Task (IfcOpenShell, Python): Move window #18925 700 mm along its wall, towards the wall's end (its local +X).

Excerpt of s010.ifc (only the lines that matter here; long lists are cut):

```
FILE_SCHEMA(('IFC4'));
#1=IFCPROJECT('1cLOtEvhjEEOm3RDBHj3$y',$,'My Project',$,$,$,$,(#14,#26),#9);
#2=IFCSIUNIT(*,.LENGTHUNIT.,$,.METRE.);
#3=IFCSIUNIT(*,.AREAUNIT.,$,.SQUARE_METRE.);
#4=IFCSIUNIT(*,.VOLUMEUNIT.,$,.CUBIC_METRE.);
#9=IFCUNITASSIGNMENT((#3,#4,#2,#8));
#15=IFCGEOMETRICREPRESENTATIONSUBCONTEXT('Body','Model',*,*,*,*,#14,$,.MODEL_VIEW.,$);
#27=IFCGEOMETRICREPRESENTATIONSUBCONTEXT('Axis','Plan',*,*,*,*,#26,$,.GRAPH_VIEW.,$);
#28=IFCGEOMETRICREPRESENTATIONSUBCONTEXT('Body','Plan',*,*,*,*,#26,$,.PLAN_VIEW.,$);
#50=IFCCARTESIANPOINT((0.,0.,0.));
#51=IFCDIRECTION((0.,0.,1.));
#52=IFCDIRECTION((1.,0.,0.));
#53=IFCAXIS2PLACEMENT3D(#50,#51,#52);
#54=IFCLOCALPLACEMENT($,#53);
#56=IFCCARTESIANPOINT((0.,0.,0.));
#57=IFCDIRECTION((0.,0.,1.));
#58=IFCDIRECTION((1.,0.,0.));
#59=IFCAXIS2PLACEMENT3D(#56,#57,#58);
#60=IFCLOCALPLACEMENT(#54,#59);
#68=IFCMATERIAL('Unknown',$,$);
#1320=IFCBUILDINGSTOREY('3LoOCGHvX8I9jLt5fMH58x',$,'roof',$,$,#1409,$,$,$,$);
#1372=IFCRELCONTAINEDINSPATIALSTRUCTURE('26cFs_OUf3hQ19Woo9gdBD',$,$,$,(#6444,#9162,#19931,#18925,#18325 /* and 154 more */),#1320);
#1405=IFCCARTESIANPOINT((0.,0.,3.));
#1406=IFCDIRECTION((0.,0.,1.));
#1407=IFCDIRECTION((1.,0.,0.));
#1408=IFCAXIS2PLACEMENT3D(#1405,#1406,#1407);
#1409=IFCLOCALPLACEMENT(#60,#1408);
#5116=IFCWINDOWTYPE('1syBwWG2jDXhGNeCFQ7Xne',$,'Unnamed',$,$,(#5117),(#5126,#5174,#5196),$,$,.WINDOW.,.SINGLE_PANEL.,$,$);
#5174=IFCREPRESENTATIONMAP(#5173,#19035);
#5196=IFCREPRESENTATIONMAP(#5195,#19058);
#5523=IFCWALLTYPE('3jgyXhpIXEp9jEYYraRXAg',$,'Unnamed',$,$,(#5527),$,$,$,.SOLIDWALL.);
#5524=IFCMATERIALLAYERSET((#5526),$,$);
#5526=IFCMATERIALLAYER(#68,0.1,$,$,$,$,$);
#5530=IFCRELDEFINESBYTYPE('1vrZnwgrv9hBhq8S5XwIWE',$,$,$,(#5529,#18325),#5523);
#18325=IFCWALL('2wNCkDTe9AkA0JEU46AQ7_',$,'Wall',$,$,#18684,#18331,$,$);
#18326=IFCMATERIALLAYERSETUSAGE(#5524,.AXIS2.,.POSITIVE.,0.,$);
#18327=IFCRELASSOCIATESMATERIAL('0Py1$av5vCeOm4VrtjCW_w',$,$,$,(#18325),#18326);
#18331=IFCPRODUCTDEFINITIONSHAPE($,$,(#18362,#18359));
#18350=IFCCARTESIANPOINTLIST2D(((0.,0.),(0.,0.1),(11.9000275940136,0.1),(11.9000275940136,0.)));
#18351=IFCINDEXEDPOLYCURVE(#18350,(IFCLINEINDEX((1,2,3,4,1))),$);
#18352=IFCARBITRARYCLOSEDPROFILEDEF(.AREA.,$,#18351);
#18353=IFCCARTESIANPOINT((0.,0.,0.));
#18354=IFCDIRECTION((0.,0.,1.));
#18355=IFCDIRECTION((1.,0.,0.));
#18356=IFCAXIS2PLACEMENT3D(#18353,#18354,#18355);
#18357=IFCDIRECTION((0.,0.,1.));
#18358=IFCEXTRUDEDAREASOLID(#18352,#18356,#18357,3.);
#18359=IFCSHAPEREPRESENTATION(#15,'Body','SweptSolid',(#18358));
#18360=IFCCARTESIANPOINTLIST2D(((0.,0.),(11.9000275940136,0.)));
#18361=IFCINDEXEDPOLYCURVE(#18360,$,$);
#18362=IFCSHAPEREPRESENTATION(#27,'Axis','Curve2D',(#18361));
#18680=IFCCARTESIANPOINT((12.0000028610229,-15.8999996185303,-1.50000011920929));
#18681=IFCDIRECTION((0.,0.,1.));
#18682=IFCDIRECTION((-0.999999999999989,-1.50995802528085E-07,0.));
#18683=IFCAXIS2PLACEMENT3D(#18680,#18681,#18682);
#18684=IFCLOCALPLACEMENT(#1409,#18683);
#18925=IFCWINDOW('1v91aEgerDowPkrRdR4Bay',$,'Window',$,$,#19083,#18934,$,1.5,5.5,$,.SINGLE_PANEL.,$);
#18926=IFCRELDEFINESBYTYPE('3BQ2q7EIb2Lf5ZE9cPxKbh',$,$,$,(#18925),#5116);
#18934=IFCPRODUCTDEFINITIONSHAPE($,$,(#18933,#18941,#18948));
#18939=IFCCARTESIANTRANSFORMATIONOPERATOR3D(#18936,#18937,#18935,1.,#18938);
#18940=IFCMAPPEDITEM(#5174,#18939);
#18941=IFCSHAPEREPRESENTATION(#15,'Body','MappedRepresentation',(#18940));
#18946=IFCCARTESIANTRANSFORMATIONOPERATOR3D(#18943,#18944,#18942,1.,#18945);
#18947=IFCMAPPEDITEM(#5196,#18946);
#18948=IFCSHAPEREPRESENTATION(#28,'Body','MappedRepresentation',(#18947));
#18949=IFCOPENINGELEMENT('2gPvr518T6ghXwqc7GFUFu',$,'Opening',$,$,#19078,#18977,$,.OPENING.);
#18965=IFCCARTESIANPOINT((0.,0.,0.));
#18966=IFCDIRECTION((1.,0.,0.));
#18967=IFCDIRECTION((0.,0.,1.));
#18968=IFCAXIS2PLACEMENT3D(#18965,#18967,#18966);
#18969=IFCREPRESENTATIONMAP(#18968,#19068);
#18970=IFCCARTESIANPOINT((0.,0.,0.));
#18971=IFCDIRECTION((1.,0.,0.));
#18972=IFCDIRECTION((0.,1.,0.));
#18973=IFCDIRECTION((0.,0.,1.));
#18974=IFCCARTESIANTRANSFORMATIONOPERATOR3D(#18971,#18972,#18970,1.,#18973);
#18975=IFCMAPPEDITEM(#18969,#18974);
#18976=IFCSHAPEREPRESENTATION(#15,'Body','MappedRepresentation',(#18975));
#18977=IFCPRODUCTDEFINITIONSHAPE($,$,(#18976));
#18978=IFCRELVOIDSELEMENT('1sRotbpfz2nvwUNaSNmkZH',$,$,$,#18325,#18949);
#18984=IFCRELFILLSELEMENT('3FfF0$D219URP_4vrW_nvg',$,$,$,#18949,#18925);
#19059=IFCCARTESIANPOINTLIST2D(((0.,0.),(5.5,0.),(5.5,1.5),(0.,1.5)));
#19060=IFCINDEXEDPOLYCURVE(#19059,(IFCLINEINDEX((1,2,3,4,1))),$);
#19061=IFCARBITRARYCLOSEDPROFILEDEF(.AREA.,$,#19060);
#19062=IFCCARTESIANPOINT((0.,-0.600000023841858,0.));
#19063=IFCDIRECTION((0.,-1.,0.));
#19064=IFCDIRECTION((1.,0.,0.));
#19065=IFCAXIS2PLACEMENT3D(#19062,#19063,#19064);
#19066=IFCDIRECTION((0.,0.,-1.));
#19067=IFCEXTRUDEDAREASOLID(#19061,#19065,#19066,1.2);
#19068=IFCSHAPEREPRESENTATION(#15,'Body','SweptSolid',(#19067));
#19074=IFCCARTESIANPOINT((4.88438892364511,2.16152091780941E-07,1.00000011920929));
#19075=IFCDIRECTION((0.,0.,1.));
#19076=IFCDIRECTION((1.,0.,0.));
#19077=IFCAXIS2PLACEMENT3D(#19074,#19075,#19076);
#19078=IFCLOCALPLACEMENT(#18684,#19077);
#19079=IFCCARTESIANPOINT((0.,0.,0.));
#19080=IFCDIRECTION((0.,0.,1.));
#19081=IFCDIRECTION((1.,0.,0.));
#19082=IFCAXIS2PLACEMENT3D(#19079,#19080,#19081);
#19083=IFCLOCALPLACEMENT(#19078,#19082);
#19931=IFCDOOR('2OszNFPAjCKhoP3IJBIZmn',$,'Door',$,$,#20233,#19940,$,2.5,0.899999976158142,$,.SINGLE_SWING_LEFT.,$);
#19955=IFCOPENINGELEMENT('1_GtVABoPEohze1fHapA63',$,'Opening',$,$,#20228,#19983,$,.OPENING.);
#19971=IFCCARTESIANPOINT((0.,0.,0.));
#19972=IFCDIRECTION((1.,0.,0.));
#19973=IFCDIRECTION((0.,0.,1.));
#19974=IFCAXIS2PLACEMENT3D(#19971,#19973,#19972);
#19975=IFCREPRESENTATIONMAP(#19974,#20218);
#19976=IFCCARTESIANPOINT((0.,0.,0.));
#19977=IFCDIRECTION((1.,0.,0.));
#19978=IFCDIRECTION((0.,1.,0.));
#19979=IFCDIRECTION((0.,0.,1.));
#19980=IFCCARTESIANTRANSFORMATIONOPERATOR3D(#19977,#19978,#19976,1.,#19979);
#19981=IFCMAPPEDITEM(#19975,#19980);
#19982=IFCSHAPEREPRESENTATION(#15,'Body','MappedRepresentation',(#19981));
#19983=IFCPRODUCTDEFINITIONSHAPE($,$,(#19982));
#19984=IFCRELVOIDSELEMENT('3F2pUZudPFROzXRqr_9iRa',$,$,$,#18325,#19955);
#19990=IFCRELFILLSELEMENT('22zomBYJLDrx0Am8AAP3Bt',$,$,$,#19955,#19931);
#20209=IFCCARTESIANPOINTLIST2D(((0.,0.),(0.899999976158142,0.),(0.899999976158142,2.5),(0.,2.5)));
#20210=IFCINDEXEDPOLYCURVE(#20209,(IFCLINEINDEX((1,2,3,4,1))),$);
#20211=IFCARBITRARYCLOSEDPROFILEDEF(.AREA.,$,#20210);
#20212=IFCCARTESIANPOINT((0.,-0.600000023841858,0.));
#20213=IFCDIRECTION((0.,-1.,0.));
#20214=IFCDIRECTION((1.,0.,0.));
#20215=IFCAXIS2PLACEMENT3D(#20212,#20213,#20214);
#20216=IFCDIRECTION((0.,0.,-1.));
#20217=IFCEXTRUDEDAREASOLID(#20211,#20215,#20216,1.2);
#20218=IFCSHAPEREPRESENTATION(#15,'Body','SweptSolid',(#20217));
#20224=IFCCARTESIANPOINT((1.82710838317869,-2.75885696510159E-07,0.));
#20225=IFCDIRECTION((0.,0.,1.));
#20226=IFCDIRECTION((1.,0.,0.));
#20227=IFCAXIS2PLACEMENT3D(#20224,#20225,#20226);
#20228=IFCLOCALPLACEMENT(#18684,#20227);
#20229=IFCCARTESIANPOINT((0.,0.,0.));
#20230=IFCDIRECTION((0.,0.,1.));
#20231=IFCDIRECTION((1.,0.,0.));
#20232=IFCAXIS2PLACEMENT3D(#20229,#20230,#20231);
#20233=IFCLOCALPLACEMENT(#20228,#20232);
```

```python
import ifcopenshell
import ifcopenshell.api.geometry
import ifcopenshell.util.placement
import ifcopenshell.util.unit

model = ifcopenshell.open("s010.ifc")
unit_scale = ifcopenshell.util.unit.calculate_unit_scale(model)

window = model.by_guid("1v91aEgerDowPkrRdR4Bay")
opening = window.FillsVoids[0].RelatingOpeningElement
wall = opening.VoidsElements[0].RelatingBuildingElement

wall_matrix = ifcopenshell.util.placement.get_local_placement(wall.ObjectPlacement)
shift = wall_matrix[:3, 0] * 0.7 / unit_scale
before = ifcopenshell.util.placement.get_local_placement(window.ObjectPlacement)[:3, 3].copy()

# The window is placed relative to its opening, so it follows when the opening moves.
matrix = ifcopenshell.util.placement.get_local_placement(opening.ObjectPlacement)
matrix[:3, 3] += shift
ifcopenshell.api.geometry.edit_object_placement(
    model, product=opening, matrix=matrix, is_si=False, should_transform_children=True
)

after = ifcopenshell.util.placement.get_local_placement(window.ObjectPlacement)[:3, 3]
print("window moved by", (after - before).round(3) + 0.0)

model.write("s010_edited.ifc")
```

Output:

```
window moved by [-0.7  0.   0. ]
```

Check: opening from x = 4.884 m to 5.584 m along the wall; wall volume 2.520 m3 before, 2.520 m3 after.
